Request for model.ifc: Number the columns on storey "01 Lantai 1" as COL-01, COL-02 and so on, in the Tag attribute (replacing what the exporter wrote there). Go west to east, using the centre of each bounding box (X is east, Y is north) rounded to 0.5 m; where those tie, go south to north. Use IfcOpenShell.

First a look at what the model holds.

```python
import ifcopenshell
import ifcopenshell.util.element
import ifcopenshell.util.placement

model = ifcopenshell.open("model.ifc")
print(model.schema)
storey = next(s for s in model.by_type("IfcBuildingStorey") if s.Name == "01 Lantai 1")
columns = [e for e in ifcopenshell.util.element.get_decomposition(storey) if e.is_a("IfcColumn")]
for e in sorted(columns, key=lambda e: e.id()):
    origin = ifcopenshell.util.placement.get_local_placement(e.ObjectPlacement)[:3, 3]
    print(e.id(), e.Tag, e.Name, origin.round(2) + 0.0, sep=" | ")
```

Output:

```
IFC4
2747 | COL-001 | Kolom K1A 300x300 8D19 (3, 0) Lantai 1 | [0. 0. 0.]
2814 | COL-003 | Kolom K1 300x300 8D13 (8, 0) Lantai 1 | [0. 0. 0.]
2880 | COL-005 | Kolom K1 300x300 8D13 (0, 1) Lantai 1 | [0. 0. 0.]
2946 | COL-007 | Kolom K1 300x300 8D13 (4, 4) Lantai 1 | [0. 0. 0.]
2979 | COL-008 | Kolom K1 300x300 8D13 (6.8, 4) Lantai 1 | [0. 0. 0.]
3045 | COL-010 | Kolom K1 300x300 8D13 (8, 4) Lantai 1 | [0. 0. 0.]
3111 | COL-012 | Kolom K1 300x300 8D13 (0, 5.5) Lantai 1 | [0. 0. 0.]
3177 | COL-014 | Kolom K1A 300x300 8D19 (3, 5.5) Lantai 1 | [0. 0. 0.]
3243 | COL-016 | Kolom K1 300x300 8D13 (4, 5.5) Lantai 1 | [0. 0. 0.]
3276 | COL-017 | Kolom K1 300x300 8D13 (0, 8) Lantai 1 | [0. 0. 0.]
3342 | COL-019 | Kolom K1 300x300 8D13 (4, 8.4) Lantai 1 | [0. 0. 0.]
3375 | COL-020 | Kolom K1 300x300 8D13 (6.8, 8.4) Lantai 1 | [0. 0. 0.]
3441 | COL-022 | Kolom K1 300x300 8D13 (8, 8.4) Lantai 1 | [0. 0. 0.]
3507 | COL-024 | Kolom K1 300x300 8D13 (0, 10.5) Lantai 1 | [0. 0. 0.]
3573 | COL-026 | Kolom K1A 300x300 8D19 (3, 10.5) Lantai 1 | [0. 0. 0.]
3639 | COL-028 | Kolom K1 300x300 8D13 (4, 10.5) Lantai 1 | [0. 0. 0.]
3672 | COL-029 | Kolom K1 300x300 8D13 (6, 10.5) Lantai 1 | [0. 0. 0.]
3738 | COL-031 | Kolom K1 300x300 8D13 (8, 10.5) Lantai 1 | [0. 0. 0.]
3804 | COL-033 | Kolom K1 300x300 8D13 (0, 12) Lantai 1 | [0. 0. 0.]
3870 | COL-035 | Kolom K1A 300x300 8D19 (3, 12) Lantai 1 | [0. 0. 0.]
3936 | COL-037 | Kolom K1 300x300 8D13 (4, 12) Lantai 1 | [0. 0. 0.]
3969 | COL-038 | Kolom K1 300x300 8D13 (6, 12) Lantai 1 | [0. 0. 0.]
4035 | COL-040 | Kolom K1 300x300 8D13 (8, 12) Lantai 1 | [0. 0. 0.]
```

```python
import ifcopenshell
import ifcopenshell.geom
import ifcopenshell.util.element
import ifcopenshell.util.shape

model = ifcopenshell.open("model.ifc")
settings = ifcopenshell.geom.settings()
settings.set("use-world-coords", True)


def centre(element):
    shape = ifcopenshell.geom.create_shape(settings, element)
    return ifcopenshell.util.shape.get_bbox_centroid(shape.geometry)


storey = next(s for s in model.by_type("IfcBuildingStorey") if s.Name == "01 Lantai 1")
columns = [e for e in ifcopenshell.util.element.get_decomposition(storey) if e.is_a("IfcColumn")]

# Insertion points can sit at a corner or the storey origin, so sort by the geometry (in metres).
centres = {e: centre(e) for e in columns}
columns.sort(key=lambda e: (round(centres[e][0] / 0.5), centres[e][1]))

for i, e in enumerate(columns, start=1):
    number = f"COL-{i:02d}"
    e.Tag = number
    print(e.id(), number)

model.write("model-out.ifc")
```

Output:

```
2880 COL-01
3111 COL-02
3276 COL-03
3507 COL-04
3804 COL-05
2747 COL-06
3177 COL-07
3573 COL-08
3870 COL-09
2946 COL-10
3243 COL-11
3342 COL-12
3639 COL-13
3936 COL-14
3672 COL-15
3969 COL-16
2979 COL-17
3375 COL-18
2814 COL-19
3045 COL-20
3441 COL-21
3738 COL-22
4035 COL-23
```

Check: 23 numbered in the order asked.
